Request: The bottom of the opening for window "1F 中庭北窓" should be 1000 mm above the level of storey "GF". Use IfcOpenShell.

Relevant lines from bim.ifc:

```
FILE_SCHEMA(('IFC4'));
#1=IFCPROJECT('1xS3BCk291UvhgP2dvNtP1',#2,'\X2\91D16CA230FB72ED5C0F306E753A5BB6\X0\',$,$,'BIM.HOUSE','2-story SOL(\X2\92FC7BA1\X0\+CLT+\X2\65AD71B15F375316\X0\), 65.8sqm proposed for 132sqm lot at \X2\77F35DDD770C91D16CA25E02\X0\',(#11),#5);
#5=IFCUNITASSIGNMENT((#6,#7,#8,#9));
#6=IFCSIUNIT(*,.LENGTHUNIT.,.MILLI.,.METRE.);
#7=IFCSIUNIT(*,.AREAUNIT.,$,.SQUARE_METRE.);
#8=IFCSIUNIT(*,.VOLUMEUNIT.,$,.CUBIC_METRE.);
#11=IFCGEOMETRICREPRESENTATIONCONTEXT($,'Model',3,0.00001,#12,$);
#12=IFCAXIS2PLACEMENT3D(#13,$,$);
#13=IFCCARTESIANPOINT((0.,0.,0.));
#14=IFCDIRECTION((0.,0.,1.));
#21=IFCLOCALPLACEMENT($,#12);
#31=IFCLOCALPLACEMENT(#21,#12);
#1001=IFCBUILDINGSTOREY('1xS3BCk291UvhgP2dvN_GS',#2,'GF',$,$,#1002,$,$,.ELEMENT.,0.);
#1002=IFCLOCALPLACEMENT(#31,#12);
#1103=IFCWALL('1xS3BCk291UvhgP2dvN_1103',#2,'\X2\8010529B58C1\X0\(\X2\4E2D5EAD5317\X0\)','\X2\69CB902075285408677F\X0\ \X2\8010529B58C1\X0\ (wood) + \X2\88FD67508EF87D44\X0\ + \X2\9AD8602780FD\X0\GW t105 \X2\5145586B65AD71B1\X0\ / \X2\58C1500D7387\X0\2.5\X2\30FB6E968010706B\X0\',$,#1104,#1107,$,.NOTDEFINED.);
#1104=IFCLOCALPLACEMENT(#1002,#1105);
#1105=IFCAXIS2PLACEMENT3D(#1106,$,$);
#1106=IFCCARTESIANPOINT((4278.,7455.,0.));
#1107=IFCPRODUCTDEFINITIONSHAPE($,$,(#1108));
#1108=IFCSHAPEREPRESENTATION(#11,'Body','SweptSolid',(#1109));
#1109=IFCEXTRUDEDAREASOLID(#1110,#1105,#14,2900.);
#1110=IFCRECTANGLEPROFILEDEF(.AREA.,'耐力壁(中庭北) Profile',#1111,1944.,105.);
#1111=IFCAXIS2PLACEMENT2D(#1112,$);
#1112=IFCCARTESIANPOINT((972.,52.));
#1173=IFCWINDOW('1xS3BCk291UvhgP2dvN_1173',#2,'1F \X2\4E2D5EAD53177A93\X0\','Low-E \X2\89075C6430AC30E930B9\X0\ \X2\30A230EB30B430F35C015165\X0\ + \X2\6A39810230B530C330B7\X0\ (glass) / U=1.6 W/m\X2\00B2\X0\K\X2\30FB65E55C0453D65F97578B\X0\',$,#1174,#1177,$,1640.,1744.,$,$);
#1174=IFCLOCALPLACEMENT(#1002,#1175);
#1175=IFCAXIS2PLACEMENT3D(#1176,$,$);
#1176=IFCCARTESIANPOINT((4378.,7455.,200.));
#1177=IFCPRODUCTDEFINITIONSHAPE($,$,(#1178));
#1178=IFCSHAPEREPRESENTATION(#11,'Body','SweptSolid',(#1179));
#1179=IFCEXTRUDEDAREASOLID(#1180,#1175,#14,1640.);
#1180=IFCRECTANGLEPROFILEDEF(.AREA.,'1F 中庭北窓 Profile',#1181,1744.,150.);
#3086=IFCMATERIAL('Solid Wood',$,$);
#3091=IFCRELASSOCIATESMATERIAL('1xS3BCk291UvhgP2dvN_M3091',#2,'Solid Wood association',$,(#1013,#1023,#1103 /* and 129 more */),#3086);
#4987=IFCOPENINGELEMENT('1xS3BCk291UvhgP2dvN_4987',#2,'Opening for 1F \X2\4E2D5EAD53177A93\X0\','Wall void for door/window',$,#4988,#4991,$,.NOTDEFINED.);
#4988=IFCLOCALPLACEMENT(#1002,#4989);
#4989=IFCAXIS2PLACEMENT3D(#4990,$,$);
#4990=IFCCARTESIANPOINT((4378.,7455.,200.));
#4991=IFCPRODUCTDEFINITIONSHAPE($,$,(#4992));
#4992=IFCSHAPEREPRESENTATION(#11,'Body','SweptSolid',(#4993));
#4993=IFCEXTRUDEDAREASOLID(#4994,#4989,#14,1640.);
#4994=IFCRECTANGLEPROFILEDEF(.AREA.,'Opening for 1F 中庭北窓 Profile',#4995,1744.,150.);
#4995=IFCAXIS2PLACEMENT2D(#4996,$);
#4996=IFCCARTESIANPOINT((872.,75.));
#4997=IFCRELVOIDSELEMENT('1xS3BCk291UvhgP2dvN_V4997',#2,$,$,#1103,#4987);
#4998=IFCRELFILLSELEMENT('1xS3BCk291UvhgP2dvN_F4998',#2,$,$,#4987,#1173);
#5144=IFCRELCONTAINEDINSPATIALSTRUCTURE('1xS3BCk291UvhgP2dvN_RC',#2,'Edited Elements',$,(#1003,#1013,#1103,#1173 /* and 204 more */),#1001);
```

```python
import numpy as np
import ifcopenshell
import ifcopenshell.api.geometry
import ifcopenshell.geom
import ifcopenshell.util.element
import ifcopenshell.util.placement
import ifcopenshell.util.shape
import ifcopenshell.util.unit

model = ifcopenshell.open("bim.ifc")
unit_scale = ifcopenshell.util.unit.calculate_unit_scale(model)

window = model.by_guid("1xS3BCk291UvhgP2dvN_1173")
opening = window.FillsVoids[0].RelatingOpeningElement
storey = ifcopenshell.util.element.get_container(window, ifc_class="IfcBuildingStorey")
level = ifcopenshell.util.placement.get_local_placement(storey.ObjectPlacement)[2, 3]

# The opening's origin need not be at the sill, so measure its lowest point.
shape = ifcopenshell.geom.create_shape(ifcopenshell.geom.settings(), opening)
bottom = ifcopenshell.util.shape.get_shape_bottom_elevation(shape, shape.geometry) / unit_scale
dz = level + 1 / unit_scale - bottom

shift = np.array([0.0, 0.0, dz])
# The window is not placed relative to its opening, so move both.
for product in (opening, window):
    matrix = ifcopenshell.util.placement.get_local_placement(product.ObjectPlacement)
    matrix[:3, 3] += shift
    ifcopenshell.api.geometry.edit_object_placement(model, product=product, matrix=matrix, is_si=False)

print(f"moved by {dz * unit_scale:+.3f} m")

model.write("bim-out.ifc")
```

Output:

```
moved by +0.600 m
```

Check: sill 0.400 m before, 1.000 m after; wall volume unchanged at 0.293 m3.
